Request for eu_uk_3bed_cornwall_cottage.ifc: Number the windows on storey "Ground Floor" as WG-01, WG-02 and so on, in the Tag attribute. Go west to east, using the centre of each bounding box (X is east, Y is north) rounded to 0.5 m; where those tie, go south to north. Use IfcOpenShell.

First a look at what the model holds.

```python
import ifcopenshell
import ifcopenshell.util.element
import ifcopenshell.util.placement

model = ifcopenshell.open("eu_uk_3bed_cornwall_cottage.ifc")
print(model.schema)
storey = next(s for s in model.by_type("IfcBuildingStorey") if s.Name == "Ground Floor")
windows = [e for e in ifcopenshell.util.element.get_decomposition(storey) if e.is_a("IfcWindow")]
for e in sorted(windows, key=lambda e: e.id()):
    origin = ifcopenshell.util.placement.get_local_placement(e.ObjectPlacement)[:3, 3]
    print(e.id(), e.Tag, e.Name, origin.round(2) + 0.0, sep=" | ")
```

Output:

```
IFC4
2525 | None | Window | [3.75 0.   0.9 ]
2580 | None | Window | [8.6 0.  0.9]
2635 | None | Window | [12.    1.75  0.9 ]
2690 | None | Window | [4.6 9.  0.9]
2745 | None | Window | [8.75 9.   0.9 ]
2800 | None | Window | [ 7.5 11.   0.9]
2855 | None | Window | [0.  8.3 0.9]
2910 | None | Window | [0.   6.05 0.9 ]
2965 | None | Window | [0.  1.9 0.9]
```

```python
import ifcopenshell
import ifcopenshell.geom
import ifcopenshell.util.element
import ifcopenshell.util.shape

model = ifcopenshell.open("eu_uk_3bed_cornwall_cottage.ifc")
settings = ifcopenshell.geom.settings()
settings.set("use-world-coords", True)


def centre(element):
    shape = ifcopenshell.geom.create_shape(settings, element)
    return ifcopenshell.util.shape.get_bbox_centroid(shape.geometry)


storey = next(s for s in model.by_type("IfcBuildingStorey") if s.Name == "Ground Floor")
windows = [e for e in ifcopenshell.util.element.get_decomposition(storey) if e.is_a("IfcWindow")]

# Insertion points can sit at a corner or the storey origin, so sort by the geometry (in metres).
centres = {e: centre(e) for e in windows}
windows.sort(key=lambda e: (round(centres[e][0] / 0.5), centres[e][1]))

for i, e in enumerate(windows, start=1):
    number = f"WG-{i:02d}"
    e.Tag = number
    print(e.id(), number)

model.write("eu_uk_3bed_cornwall_cottage_updated.ifc")
```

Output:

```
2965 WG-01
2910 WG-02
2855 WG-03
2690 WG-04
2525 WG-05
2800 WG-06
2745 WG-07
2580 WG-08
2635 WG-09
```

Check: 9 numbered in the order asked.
